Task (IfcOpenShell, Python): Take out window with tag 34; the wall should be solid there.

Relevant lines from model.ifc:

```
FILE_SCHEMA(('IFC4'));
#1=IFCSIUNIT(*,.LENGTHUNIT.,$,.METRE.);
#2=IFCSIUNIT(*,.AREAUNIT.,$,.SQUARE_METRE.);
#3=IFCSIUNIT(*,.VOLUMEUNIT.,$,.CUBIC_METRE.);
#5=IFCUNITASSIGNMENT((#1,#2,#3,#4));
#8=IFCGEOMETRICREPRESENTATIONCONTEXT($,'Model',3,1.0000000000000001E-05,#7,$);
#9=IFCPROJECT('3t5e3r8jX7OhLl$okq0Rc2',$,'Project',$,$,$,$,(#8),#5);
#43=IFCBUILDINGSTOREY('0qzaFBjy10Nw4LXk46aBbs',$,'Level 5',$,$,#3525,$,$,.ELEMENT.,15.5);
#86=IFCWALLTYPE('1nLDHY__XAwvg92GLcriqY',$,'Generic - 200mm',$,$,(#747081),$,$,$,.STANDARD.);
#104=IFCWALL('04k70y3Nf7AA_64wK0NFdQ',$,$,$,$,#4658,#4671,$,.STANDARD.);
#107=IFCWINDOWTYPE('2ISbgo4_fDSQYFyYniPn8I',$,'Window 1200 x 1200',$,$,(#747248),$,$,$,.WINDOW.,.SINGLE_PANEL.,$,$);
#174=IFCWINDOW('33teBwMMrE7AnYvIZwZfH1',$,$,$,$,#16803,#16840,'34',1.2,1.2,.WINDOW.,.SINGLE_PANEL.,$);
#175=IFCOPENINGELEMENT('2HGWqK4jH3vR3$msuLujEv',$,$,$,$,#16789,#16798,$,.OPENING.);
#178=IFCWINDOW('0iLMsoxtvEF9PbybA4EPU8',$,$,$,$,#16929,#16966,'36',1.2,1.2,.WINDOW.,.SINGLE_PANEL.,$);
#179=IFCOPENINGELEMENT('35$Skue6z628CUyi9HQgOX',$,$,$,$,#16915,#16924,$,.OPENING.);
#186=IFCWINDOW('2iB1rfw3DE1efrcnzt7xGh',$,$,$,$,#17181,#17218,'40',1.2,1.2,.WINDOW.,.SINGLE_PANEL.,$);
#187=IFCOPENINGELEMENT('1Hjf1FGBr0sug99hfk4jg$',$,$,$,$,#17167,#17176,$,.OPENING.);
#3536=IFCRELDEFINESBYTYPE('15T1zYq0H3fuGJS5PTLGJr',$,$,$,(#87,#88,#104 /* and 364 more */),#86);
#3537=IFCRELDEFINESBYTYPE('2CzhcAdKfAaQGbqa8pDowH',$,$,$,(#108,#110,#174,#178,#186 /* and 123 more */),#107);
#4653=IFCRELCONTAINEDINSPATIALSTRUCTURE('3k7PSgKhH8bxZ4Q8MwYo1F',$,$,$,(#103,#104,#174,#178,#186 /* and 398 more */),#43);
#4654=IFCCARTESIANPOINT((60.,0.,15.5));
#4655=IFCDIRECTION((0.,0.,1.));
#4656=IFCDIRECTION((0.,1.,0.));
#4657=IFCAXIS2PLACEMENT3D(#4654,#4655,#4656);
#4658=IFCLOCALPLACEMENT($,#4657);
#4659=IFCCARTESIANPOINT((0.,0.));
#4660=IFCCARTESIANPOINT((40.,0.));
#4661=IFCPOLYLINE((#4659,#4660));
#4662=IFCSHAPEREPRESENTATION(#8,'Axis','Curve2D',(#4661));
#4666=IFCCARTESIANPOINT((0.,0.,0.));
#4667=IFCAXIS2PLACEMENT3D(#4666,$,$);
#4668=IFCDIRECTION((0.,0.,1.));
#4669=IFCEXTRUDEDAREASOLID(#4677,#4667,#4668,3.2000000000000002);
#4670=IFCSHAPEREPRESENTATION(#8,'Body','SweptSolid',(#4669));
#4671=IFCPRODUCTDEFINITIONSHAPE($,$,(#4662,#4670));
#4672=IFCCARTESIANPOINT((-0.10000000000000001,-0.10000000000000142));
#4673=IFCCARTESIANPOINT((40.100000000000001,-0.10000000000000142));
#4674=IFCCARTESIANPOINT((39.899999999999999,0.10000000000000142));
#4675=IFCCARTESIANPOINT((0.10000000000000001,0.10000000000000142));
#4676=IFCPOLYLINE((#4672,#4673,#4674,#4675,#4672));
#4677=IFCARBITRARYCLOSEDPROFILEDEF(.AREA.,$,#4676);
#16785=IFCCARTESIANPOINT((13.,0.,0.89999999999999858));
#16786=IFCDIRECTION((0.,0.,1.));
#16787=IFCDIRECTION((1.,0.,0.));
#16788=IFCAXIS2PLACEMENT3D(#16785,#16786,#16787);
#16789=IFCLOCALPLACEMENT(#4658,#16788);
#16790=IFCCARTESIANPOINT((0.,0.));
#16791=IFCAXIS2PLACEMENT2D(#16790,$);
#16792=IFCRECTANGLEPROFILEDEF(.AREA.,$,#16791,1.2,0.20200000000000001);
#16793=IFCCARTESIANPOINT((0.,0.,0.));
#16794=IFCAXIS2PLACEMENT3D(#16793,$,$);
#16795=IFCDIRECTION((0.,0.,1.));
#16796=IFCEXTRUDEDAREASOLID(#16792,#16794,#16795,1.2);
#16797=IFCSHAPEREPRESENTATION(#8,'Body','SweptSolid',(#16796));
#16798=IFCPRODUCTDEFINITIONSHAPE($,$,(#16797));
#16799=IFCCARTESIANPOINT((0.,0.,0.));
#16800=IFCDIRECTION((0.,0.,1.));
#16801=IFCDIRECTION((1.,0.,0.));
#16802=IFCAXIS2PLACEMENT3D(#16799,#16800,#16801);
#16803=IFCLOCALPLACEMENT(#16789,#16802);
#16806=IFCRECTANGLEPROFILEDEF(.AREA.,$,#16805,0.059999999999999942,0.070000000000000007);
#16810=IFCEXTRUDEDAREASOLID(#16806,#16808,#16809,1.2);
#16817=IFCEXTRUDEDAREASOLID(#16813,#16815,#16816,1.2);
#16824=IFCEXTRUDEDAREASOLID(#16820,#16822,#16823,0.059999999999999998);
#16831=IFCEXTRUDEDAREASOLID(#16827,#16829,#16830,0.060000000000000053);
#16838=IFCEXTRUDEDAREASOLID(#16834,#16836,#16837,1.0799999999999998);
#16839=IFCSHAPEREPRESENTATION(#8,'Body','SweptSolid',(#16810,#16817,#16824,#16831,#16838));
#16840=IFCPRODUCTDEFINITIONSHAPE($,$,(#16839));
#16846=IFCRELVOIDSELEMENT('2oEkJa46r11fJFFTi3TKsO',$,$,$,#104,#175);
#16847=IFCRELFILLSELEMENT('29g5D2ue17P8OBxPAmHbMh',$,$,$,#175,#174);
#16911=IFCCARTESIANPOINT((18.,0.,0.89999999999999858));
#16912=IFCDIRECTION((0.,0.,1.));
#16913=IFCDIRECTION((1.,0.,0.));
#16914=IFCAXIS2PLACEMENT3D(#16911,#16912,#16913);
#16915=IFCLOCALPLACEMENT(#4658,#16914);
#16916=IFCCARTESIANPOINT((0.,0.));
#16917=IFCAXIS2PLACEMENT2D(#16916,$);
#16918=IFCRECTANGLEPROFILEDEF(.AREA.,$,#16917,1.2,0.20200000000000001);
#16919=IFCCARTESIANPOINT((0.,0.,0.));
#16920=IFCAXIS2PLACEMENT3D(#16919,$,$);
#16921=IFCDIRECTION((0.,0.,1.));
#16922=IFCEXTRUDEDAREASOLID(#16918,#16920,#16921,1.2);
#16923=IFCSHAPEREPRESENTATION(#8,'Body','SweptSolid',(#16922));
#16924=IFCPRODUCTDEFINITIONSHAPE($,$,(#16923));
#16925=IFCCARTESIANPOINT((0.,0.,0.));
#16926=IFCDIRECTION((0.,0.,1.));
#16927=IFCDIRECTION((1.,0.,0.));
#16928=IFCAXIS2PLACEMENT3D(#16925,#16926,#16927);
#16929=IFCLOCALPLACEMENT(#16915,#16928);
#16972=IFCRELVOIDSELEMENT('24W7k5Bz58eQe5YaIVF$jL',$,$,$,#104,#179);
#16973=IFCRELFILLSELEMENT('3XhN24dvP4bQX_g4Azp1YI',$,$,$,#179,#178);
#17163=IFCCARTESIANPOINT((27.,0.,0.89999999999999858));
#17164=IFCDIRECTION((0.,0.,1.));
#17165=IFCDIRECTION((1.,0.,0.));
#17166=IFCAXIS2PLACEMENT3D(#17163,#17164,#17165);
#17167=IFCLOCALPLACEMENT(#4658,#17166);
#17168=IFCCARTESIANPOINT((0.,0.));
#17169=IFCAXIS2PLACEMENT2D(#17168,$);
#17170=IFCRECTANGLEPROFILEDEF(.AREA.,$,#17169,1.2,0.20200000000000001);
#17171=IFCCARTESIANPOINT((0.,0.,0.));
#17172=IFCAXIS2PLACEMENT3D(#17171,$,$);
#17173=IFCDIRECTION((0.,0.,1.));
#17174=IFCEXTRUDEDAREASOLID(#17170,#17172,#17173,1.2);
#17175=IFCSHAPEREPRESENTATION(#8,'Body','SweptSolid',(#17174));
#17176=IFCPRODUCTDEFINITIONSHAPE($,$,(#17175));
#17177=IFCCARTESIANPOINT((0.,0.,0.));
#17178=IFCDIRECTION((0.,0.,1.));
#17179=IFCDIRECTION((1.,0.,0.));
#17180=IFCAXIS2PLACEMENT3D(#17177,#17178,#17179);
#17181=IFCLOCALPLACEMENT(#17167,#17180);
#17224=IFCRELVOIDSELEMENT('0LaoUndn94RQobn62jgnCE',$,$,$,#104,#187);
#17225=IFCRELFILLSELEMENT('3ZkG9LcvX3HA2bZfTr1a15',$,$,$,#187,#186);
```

```python
import ifcopenshell
import ifcopenshell.api.feature
import ifcopenshell.api.root
import ifcopenshell.geom
import ifcopenshell.util.shape

model = ifcopenshell.open("model.ifc")
settings = ifcopenshell.geom.settings()


def volume(element):
    """Net volume in cubic metres, openings subtracted."""
    shape = ifcopenshell.geom.create_shape(settings, element)
    return ifcopenshell.util.shape.get_volume(shape.geometry)


window = model.by_guid("33teBwMMrE7AnYvIZwZfH1")
opening = window.FillsVoids[0].RelatingOpeningElement
wall = opening.VoidsElements[0].RelatingBuildingElement
before = volume(wall)

ifcopenshell.api.root.remove_product(model, product=window)
ifcopenshell.api.feature.remove_feature(model, feature=opening)

after = volume(wall)

print(f"wall volume {before:.3f} -> {after:.3f} m3")

model.write("model-out.ifc")
```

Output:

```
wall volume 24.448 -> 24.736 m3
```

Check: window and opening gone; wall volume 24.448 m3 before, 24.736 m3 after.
